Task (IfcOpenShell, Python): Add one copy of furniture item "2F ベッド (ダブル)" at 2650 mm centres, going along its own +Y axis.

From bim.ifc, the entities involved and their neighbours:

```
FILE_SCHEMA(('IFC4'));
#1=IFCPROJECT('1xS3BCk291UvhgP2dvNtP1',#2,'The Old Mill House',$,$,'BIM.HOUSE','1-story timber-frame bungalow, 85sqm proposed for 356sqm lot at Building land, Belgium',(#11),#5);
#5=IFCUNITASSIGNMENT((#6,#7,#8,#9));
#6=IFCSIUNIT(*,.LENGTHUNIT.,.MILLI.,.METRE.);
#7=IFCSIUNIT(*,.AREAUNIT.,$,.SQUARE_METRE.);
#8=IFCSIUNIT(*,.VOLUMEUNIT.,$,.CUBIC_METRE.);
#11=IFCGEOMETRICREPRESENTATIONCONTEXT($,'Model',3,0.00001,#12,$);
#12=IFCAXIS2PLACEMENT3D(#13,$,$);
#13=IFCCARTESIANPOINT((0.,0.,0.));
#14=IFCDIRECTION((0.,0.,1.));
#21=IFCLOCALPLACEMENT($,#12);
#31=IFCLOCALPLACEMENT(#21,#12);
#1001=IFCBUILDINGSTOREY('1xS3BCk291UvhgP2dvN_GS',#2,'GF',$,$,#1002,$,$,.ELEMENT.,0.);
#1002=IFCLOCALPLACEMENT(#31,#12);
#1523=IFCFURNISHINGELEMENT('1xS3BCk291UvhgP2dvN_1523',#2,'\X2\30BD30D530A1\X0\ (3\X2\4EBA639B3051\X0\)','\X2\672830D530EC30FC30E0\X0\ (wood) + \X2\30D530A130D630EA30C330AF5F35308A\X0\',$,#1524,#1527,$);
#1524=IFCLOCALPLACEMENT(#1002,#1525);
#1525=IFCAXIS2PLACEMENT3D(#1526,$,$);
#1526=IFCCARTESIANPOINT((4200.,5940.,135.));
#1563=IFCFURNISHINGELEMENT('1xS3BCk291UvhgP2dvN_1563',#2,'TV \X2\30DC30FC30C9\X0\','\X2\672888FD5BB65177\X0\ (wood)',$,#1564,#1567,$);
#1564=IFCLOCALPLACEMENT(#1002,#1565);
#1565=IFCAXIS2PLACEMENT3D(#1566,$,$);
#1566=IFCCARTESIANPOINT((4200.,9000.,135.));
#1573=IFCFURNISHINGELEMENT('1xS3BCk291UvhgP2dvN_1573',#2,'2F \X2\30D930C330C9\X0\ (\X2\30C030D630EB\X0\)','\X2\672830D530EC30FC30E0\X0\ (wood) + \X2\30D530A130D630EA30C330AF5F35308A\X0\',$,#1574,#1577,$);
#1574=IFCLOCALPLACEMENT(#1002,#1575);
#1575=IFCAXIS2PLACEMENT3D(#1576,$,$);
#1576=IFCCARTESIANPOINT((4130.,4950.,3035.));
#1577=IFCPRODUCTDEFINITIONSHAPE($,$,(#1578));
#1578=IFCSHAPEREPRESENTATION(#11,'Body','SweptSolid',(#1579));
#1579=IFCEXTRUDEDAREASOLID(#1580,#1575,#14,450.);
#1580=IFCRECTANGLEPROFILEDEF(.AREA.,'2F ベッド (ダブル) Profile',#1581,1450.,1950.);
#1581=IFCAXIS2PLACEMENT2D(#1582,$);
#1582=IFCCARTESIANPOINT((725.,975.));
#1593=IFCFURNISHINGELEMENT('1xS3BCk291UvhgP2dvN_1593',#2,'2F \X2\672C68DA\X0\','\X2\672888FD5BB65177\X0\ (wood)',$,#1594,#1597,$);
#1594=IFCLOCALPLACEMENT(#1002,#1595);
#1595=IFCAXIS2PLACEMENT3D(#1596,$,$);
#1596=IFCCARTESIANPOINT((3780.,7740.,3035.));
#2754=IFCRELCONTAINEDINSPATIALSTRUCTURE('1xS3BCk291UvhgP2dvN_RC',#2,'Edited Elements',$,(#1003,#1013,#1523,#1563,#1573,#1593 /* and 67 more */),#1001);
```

```python
import ifcopenshell
import ifcopenshell.api.geometry
import ifcopenshell.api.root
import ifcopenshell.util.element
import ifcopenshell.util.placement
import ifcopenshell.util.unit

model = ifcopenshell.open("bim.ifc")
unit_scale = ifcopenshell.util.unit.calculate_unit_scale(model)


def reuse_history(source, copy):
    """copy_class also copies each property set's owner history, people and application; keep the originals."""
    for rel in copy.IsDefinedBy:
        if rel.is_a("IfcRelDefinesByProperties") and (history := rel.RelatingPropertyDefinition.OwnerHistory):
            rel.RelatingPropertyDefinition.OwnerHistory = source.OwnerHistory
            ifcopenshell.util.element.remove_deep2(model, history)


source = model.by_guid("1xS3BCk291UvhgP2dvN_1573")
base = ifcopenshell.util.placement.get_local_placement(source.ObjectPlacement)
step = base[:3, 1] * 2.65 / unit_scale

for i in range(1, 2):
    copy = ifcopenshell.api.root.copy_class(model, product=source)
    copy.Representation = ifcopenshell.util.element.copy_deep(
        model, source.Representation, exclude=["IfcGeometricRepresentationContext", "IfcRepresentationMap"]
    )
    reuse_history(source, copy)
    matrix = base.copy()
    matrix[:3, 3] += i * step
    print("added at", matrix[:3, 3].round(3) + 0.0)
    ifcopenshell.api.geometry.edit_object_placement(model, product=copy, matrix=matrix, is_si=False)

model.write("bim_edited.ifc")
```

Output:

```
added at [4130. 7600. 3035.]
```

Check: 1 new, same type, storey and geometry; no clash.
